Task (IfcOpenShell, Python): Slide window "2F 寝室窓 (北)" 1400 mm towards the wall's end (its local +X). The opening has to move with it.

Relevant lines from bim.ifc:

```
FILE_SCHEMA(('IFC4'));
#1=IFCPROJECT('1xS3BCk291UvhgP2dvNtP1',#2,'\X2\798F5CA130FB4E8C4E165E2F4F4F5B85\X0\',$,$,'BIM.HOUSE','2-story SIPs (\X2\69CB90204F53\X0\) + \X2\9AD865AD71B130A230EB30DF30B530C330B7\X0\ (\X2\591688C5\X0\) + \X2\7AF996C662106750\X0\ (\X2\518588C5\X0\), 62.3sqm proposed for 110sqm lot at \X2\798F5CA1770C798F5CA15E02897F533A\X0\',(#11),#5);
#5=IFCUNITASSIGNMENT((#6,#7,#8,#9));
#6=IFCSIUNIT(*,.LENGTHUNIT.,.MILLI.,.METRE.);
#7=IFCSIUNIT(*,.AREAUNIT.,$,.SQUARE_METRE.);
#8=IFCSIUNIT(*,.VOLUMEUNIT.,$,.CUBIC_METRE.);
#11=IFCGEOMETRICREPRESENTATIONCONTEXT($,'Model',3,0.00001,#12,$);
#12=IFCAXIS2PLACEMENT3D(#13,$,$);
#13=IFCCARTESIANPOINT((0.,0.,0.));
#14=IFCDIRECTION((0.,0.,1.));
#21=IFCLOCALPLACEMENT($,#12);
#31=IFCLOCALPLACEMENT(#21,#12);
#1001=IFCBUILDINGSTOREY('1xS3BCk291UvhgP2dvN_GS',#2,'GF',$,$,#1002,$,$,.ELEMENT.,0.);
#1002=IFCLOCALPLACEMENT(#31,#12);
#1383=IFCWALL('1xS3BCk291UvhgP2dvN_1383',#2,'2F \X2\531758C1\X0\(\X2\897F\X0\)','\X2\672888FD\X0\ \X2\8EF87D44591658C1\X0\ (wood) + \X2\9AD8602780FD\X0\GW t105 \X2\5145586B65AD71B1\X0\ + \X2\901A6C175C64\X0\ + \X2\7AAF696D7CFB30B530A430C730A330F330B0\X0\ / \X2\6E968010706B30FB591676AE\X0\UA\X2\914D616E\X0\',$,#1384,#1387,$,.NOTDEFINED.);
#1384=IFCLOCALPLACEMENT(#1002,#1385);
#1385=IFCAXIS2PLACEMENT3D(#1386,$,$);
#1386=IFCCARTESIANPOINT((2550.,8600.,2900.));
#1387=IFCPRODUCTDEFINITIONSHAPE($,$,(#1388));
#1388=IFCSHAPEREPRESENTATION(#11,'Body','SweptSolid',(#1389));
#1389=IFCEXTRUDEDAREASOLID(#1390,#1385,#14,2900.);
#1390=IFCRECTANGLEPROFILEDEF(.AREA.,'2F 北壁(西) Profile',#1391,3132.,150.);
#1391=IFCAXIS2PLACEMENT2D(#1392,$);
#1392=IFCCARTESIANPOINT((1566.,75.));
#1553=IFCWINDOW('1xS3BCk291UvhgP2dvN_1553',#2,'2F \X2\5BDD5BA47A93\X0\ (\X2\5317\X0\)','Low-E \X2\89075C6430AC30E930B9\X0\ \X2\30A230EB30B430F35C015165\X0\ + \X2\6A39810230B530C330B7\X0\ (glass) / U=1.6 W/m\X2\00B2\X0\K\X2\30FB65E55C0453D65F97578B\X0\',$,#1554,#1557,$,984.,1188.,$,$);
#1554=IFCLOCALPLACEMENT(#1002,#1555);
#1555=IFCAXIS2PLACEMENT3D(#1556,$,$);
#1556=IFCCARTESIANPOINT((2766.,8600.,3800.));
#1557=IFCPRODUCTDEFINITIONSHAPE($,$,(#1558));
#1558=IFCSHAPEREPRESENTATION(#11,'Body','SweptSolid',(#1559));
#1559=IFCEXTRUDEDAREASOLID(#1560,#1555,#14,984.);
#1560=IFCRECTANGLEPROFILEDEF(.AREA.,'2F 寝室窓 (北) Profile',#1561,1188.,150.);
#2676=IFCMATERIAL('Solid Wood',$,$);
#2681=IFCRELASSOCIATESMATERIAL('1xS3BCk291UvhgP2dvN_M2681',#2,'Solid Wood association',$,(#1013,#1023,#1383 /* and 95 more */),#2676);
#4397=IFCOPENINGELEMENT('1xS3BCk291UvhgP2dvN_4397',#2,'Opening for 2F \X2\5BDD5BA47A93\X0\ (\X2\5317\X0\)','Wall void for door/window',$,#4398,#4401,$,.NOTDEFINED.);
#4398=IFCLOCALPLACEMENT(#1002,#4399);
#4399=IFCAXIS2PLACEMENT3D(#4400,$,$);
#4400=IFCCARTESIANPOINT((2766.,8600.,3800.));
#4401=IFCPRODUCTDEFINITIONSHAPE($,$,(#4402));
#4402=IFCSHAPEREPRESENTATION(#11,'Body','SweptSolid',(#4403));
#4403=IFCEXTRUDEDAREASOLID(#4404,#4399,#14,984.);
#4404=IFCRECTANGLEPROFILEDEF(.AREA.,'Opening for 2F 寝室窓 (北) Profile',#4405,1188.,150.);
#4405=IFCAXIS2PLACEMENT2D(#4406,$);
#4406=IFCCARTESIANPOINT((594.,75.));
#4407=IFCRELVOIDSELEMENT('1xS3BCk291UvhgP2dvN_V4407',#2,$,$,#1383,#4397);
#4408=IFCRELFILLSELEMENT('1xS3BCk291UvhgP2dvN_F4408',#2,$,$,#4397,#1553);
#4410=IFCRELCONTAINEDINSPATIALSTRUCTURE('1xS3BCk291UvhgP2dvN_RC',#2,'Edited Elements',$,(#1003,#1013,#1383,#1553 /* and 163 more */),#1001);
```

```python
import ifcopenshell
import ifcopenshell.api.geometry
import ifcopenshell.util.placement

model = ifcopenshell.open("bim.ifc")

window = model.by_guid("1xS3BCk291UvhgP2dvN_1553")
opening = window.FillsVoids[0].RelatingOpeningElement
wall = opening.VoidsElements[0].RelatingBuildingElement

wall_matrix = ifcopenshell.util.placement.get_local_placement(wall.ObjectPlacement)
shift = wall_matrix[:3, 0] * 1400.0
before = ifcopenshell.util.placement.get_local_placement(window.ObjectPlacement)[:3, 3].copy()

# The window is not placed relative to its opening, so move both.
for product in (opening, window):
    matrix = ifcopenshell.util.placement.get_local_placement(product.ObjectPlacement)
    matrix[:3, 3] += shift
    ifcopenshell.api.geometry.edit_object_placement(model, product=product, matrix=matrix, is_si=False)

after = ifcopenshell.util.placement.get_local_placement(window.ObjectPlacement)[:3, 3]
print("window moved by", (after - before).round(3) + 0.0)

model.write("bim_v2.ifc")
```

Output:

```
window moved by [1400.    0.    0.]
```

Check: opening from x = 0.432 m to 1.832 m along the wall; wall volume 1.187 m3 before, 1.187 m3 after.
